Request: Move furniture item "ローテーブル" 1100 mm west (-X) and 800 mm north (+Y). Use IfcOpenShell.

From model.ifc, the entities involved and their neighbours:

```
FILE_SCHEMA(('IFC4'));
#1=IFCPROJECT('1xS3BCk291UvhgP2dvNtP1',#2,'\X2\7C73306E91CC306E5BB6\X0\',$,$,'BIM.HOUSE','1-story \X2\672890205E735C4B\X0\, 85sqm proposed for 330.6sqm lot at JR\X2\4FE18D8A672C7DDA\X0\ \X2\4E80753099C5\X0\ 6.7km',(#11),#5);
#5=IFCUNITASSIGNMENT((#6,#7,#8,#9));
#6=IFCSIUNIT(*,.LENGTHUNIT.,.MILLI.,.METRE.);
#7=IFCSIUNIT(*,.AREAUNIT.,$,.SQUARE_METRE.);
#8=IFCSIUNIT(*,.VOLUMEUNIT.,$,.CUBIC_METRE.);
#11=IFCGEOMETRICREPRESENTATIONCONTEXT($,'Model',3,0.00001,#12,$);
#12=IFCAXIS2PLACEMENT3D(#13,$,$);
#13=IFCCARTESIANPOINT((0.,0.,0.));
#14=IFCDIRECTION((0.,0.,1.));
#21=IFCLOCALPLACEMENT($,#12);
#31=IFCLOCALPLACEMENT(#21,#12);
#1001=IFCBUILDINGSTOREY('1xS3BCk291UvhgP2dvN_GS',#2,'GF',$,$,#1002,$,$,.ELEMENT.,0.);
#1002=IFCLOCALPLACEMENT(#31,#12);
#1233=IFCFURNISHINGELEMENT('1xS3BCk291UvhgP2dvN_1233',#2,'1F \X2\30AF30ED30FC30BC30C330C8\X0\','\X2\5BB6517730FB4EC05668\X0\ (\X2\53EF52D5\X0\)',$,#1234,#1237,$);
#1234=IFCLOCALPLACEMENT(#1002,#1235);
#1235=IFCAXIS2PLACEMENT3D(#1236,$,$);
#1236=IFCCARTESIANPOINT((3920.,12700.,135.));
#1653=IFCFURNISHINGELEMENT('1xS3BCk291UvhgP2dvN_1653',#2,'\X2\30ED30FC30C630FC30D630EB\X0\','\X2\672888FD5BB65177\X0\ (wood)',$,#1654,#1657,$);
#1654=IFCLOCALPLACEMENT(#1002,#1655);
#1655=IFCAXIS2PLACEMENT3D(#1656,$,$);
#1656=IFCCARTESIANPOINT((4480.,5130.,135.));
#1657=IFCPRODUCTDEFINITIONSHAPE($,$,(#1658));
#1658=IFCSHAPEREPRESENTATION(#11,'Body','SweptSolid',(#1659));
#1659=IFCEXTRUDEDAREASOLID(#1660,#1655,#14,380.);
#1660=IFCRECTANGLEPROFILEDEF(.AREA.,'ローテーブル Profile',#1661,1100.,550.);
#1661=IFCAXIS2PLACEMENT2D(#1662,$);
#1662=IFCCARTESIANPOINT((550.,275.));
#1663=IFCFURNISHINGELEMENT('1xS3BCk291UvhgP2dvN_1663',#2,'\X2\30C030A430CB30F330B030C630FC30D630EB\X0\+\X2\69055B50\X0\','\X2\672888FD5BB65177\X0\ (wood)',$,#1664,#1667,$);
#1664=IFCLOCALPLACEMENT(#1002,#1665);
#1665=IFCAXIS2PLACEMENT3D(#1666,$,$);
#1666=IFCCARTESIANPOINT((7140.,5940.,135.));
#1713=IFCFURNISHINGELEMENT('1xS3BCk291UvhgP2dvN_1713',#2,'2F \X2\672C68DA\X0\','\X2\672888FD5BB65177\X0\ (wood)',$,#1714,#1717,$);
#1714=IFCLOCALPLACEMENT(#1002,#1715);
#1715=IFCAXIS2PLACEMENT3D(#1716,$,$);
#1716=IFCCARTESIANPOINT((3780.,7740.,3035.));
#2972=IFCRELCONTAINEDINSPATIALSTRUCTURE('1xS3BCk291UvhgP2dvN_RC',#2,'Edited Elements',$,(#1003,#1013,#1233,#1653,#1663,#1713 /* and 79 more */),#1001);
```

```python
import ifcopenshell
import ifcopenshell.api.geometry
import ifcopenshell.util.placement
import ifcopenshell.util.unit

model = ifcopenshell.open("model.ifc")
unit_scale = ifcopenshell.util.unit.calculate_unit_scale(model)

item = model.by_id(1653)
matrix = ifcopenshell.util.placement.get_local_placement(item.ObjectPlacement)
matrix[0, 3] -= 1.1 / unit_scale
matrix[1, 3] += 0.8 / unit_scale
ifcopenshell.api.geometry.edit_object_placement(model, product=item, matrix=matrix, is_si=False)

print(ifcopenshell.util.placement.get_local_placement(item.ObjectPlacement).round(3) + 0.0)

model.write("model_rev.ifc")
```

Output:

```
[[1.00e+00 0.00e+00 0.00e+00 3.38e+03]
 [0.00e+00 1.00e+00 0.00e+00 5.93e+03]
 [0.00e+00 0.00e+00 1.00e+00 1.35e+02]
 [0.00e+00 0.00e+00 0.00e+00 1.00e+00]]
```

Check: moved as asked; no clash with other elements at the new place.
